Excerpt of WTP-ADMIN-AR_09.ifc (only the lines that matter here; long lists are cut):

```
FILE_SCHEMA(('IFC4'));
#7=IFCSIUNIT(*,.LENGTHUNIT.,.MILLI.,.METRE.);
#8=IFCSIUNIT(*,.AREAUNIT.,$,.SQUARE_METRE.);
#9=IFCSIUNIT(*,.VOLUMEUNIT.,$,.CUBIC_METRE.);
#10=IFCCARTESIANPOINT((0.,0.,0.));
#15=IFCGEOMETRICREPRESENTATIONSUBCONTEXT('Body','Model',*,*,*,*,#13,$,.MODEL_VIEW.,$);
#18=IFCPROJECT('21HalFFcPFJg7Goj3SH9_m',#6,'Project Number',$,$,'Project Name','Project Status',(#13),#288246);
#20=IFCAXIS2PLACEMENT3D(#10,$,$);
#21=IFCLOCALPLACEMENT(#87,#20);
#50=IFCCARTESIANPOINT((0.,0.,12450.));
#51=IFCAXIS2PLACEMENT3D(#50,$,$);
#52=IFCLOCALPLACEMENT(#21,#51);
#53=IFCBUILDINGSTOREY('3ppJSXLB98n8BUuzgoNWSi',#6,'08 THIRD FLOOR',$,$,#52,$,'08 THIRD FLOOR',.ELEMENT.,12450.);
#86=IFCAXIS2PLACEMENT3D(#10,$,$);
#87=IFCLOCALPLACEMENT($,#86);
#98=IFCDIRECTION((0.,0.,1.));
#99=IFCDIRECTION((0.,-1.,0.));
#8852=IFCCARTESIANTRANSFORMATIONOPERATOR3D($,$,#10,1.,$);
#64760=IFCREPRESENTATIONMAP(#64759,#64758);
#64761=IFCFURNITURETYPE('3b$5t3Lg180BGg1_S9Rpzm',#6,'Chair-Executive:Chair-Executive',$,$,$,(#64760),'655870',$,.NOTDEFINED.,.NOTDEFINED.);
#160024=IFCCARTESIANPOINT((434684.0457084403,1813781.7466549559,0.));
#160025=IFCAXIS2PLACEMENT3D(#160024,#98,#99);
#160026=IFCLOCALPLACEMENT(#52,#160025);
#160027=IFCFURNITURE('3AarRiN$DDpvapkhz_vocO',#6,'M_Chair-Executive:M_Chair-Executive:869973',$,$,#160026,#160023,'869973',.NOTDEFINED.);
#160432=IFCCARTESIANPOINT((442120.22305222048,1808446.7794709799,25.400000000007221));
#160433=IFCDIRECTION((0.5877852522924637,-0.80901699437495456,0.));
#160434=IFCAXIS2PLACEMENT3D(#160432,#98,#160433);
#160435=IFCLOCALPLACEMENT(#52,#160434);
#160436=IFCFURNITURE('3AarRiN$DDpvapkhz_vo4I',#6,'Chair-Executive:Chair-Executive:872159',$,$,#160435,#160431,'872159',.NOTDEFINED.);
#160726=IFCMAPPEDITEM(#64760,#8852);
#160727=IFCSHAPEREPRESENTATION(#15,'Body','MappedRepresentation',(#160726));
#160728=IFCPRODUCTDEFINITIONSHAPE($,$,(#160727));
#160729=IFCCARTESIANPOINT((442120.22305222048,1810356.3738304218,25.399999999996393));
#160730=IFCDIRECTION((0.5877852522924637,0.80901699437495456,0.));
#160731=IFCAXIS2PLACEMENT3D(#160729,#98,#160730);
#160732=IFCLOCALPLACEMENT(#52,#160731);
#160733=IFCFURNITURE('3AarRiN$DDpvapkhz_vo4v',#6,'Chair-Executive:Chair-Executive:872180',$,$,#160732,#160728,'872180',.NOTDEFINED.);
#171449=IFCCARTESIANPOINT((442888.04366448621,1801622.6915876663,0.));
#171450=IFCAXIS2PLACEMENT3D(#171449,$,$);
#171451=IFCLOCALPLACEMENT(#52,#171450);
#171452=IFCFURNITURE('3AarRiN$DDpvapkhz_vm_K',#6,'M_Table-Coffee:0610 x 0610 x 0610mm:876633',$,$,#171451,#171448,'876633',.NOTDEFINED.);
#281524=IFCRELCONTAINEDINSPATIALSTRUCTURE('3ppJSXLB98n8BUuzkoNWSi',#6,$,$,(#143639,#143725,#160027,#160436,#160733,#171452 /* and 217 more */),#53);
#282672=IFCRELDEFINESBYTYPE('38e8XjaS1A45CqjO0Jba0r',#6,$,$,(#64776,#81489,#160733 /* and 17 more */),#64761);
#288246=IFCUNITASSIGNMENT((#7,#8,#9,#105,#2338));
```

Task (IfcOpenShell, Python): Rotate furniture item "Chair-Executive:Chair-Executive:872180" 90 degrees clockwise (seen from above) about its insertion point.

```python
import ifcopenshell
import ifcopenshell.api.geometry
import ifcopenshell.util.placement

model = ifcopenshell.open("WTP-ADMIN-AR_09.ifc")

item = model.by_guid("3AarRiN$DDpvapkhz_vo4v")
matrix = ifcopenshell.util.placement.get_local_placement(item.ObjectPlacement)
matrix = matrix @ ifcopenshell.util.placement.rotation(-90, "Z")
ifcopenshell.api.geometry.edit_object_placement(model, product=item, matrix=matrix, is_si=False)

print(ifcopenshell.util.placement.get_local_placement(item.ObjectPlacement).round(3) + 0.0)

model.write("WTP-ADMIN-AR_09_v2.ifc")
```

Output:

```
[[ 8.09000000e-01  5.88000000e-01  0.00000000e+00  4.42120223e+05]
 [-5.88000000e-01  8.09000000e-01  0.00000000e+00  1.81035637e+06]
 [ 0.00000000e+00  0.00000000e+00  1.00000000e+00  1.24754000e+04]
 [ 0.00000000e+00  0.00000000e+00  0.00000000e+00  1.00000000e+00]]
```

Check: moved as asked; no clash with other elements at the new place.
